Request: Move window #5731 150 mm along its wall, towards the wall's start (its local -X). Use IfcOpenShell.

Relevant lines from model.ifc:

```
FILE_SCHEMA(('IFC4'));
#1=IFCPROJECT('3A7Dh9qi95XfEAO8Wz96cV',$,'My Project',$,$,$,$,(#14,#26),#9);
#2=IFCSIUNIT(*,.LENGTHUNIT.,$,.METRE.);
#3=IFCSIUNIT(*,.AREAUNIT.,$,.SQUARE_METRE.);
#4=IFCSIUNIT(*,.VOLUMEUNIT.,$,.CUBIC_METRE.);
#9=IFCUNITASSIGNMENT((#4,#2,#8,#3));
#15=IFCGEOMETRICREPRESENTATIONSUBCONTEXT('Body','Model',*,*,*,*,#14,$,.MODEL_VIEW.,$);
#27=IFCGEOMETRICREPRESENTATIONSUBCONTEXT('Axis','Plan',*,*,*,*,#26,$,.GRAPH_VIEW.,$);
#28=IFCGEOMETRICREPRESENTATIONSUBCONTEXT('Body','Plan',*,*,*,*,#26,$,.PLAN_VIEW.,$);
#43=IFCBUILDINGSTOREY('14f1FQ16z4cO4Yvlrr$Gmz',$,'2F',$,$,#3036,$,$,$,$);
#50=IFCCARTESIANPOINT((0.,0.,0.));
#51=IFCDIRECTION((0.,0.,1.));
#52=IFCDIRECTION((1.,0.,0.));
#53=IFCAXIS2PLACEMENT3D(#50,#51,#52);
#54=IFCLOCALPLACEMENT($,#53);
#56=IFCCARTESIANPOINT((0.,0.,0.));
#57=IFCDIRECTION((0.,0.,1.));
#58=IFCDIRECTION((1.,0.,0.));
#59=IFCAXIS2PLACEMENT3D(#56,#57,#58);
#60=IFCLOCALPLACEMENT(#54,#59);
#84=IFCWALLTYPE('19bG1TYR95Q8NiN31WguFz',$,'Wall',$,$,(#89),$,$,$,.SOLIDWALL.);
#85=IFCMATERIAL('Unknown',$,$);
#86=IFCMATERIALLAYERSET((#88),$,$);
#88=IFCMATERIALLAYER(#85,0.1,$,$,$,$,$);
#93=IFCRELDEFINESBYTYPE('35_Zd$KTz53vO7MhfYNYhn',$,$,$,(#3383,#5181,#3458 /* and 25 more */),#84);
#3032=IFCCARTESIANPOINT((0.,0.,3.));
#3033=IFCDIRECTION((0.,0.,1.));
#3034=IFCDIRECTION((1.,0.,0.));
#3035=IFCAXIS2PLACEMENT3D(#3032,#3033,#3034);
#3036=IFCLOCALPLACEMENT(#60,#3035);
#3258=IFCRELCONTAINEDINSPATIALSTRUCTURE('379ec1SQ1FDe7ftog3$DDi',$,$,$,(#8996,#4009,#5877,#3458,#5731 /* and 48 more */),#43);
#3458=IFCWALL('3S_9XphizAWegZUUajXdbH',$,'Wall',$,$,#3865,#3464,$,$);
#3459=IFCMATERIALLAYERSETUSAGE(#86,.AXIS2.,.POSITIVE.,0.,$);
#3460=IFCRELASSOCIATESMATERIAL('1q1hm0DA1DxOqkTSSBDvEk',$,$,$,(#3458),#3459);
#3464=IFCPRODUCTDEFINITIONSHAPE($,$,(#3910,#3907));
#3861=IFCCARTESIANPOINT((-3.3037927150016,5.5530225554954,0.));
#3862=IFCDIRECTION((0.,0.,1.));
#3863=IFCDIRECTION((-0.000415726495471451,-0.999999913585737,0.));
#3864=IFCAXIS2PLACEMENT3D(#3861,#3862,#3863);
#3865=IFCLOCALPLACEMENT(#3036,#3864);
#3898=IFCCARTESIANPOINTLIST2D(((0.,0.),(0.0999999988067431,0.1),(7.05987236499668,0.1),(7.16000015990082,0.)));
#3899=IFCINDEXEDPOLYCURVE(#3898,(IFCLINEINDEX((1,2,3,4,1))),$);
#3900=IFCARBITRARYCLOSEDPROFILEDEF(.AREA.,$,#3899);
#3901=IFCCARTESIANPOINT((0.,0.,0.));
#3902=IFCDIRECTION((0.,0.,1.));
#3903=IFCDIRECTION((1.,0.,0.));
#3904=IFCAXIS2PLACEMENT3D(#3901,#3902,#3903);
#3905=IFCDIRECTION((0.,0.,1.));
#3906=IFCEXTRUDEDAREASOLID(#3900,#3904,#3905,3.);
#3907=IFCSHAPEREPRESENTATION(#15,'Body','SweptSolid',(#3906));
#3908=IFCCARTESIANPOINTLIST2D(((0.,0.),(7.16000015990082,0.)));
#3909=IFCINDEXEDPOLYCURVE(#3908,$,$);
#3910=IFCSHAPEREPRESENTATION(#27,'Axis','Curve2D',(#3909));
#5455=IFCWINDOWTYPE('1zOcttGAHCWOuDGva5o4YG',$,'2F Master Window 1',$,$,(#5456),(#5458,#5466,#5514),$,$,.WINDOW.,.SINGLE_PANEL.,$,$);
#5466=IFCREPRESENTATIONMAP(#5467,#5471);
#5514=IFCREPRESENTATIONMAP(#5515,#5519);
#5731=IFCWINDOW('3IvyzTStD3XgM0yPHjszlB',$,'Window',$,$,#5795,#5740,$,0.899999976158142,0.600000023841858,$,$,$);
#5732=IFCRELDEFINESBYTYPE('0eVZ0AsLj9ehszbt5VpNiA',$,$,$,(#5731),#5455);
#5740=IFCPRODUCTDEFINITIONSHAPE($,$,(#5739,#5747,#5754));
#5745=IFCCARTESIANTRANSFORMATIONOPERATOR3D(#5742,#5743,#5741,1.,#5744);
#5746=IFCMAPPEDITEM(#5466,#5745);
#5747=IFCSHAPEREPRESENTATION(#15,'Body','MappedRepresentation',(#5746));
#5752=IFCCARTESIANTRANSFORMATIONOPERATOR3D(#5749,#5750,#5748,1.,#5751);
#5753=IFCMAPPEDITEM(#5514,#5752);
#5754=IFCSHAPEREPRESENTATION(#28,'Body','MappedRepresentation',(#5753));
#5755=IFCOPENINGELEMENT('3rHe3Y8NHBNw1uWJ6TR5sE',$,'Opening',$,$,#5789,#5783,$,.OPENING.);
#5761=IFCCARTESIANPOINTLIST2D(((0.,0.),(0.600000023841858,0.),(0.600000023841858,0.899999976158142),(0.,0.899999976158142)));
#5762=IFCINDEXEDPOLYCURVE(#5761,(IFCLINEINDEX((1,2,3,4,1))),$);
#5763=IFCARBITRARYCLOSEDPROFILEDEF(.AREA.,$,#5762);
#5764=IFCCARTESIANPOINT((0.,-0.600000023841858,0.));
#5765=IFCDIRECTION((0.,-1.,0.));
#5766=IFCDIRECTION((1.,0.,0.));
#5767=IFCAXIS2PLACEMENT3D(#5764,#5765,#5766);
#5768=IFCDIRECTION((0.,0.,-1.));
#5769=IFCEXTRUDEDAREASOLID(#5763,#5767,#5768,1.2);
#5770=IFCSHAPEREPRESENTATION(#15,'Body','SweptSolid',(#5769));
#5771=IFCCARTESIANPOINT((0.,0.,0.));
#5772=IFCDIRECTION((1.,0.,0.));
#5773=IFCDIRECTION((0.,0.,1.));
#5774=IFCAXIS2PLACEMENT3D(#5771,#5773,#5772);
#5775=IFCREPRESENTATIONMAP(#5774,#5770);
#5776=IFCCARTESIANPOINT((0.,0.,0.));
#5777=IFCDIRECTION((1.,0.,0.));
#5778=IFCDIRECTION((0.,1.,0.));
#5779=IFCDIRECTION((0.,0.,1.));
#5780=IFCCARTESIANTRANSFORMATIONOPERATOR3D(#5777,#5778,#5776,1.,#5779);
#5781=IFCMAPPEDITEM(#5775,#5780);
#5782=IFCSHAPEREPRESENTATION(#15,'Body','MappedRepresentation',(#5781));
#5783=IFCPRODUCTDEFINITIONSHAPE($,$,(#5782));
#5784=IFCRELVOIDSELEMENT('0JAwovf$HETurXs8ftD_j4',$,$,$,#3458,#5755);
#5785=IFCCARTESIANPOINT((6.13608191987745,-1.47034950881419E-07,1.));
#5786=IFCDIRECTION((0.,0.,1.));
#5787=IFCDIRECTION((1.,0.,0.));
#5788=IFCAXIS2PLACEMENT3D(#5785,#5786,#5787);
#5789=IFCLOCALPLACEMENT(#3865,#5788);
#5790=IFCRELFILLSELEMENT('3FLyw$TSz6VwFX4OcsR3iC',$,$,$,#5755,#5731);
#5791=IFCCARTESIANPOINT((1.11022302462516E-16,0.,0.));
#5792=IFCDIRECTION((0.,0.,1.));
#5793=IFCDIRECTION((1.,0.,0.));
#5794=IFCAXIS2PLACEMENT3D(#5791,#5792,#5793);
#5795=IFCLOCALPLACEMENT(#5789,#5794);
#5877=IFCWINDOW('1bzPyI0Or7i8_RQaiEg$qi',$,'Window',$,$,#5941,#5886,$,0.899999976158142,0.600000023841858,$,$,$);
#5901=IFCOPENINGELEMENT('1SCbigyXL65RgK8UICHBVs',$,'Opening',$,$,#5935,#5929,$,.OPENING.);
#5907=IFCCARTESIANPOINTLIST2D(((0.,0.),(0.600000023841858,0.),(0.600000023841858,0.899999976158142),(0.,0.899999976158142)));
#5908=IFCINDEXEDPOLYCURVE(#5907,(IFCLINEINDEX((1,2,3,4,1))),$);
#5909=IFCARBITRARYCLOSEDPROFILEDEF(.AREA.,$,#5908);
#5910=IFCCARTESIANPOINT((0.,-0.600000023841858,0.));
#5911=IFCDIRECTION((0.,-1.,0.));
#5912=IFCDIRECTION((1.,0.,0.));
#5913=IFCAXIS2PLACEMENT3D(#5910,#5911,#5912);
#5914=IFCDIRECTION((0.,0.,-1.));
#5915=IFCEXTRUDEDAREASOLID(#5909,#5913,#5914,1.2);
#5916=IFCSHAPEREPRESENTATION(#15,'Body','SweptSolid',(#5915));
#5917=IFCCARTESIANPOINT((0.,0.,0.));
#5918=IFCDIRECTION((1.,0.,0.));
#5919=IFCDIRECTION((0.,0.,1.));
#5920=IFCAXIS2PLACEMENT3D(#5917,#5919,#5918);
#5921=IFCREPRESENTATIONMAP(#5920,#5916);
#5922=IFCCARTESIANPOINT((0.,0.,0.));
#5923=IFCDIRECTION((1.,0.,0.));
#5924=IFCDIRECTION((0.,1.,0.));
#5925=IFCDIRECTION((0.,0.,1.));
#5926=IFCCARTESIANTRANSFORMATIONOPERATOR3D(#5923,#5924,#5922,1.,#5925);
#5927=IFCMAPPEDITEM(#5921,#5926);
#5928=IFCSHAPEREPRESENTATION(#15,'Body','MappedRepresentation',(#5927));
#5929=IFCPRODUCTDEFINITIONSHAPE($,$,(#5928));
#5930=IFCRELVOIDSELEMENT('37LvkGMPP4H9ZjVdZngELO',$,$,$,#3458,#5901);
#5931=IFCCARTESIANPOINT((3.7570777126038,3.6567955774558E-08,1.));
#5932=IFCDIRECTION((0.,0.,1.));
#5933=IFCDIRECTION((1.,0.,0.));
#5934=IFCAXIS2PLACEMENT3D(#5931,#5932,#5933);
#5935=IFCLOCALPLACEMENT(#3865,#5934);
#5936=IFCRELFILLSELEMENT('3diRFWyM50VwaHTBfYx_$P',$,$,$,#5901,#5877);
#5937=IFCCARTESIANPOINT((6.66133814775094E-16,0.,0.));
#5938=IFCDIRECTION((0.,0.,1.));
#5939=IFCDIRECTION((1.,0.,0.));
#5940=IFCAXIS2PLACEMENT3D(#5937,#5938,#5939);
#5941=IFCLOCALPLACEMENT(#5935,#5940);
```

```python
import ifcopenshell
import ifcopenshell.api.geometry
import ifcopenshell.util.placement

model = ifcopenshell.open("model.ifc")

window = model.by_guid("3IvyzTStD3XgM0yPHjszlB")
opening = window.FillsVoids[0].RelatingOpeningElement
wall = opening.VoidsElements[0].RelatingBuildingElement

wall_matrix = ifcopenshell.util.placement.get_local_placement(wall.ObjectPlacement)
shift = wall_matrix[:3, 0] * -0.15
before = ifcopenshell.util.placement.get_local_placement(window.ObjectPlacement)[:3, 3].copy()

# The window is placed relative to its opening, so it follows when the opening moves.
matrix = ifcopenshell.util.placement.get_local_placement(opening.ObjectPlacement)
matrix[:3, 3] += shift
ifcopenshell.api.geometry.edit_object_placement(
    model, product=opening, matrix=matrix, is_si=False, should_transform_children=True
)

after = ifcopenshell.util.placement.get_local_placement(window.ObjectPlacement)[:3, 3]
print("window moved by", (after - before).round(3) + 0.0)

model.write("model_edited.ifc")
```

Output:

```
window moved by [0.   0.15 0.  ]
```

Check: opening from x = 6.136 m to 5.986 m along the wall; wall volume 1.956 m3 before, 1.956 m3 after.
